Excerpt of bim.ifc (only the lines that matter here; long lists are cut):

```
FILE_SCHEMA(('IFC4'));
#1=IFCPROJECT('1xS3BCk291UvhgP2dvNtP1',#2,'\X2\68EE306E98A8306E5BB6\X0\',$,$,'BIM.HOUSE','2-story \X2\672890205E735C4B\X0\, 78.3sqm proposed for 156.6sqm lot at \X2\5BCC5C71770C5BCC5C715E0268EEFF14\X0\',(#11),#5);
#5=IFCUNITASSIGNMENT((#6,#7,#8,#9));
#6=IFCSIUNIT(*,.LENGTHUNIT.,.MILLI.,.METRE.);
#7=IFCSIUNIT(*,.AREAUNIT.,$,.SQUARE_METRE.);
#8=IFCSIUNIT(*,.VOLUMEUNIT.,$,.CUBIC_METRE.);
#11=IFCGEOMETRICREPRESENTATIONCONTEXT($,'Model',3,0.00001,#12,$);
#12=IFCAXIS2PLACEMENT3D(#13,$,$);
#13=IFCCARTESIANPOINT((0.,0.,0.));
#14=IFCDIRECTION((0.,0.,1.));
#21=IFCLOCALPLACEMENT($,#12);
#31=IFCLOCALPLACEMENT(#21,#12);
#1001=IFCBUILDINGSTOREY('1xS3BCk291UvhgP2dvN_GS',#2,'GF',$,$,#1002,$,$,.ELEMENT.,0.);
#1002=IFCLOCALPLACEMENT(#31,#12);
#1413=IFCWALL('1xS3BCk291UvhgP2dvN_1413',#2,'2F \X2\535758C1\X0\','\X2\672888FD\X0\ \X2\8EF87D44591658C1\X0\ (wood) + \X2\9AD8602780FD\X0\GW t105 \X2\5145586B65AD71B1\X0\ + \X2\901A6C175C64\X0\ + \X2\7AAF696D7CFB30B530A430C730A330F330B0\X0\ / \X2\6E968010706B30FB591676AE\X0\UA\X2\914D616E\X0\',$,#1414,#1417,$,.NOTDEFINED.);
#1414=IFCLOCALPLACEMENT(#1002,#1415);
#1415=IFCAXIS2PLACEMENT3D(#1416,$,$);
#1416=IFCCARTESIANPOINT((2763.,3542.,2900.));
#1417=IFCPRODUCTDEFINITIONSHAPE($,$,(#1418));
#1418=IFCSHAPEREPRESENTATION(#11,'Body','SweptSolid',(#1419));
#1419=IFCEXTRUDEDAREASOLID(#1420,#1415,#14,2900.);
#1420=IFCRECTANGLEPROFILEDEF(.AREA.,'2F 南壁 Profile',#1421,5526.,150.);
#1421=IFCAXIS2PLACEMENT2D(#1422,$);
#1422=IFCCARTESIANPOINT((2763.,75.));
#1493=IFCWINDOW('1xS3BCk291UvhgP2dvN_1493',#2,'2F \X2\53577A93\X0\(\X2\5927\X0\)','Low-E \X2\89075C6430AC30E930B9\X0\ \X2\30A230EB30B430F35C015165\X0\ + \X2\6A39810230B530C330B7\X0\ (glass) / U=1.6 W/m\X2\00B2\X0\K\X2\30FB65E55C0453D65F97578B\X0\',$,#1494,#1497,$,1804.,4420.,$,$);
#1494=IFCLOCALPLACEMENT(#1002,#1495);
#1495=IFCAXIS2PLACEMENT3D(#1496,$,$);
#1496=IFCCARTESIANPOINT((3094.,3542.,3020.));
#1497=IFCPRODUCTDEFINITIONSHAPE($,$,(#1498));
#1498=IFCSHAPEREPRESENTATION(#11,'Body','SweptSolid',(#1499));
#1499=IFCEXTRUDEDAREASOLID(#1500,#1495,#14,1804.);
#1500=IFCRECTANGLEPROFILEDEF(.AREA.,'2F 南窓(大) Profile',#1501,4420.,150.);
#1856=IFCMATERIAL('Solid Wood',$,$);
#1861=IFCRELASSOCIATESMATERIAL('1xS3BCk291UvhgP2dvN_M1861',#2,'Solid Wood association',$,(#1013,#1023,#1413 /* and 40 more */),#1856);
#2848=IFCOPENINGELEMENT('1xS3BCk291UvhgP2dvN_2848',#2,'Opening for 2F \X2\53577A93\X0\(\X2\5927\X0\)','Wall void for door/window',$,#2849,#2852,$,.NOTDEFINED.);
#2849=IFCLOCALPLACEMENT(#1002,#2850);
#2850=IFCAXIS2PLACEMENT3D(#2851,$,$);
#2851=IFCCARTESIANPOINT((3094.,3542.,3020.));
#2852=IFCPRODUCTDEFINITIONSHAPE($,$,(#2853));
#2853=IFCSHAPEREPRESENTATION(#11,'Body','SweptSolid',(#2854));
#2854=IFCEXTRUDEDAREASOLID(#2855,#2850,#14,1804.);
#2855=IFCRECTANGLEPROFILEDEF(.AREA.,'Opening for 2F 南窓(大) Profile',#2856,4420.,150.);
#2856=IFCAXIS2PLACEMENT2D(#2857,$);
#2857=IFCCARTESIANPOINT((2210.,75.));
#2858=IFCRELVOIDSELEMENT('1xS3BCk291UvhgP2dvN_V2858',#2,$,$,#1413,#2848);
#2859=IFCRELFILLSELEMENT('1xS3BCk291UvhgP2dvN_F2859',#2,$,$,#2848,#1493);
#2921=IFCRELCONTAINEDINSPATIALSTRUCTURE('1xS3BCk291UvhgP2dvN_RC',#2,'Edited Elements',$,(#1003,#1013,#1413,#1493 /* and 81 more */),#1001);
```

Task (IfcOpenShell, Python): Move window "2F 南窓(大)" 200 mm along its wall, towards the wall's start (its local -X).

```python
import ifcopenshell
import ifcopenshell.api.geometry
import ifcopenshell.util.placement

model = ifcopenshell.open("bim.ifc")

window = model.by_guid("1xS3BCk291UvhgP2dvN_1493")
opening = window.FillsVoids[0].RelatingOpeningElement
wall = opening.VoidsElements[0].RelatingBuildingElement

wall_matrix = ifcopenshell.util.placement.get_local_placement(wall.ObjectPlacement)
shift = wall_matrix[:3, 0] * -200.0
before = ifcopenshell.util.placement.get_local_placement(window.ObjectPlacement)[:3, 3].copy()

# The window is not placed relative to its opening, so move both.
for product in (opening, window):
    matrix = ifcopenshell.util.placement.get_local_placement(product.ObjectPlacement)
    matrix[:3, 3] += shift
    ifcopenshell.api.geometry.edit_object_placement(model, product=product, matrix=matrix, is_si=False)

after = ifcopenshell.util.placement.get_local_placement(window.ObjectPlacement)[:3, 3]
print("window moved by", (after - before).round(3) + 0.0)

model.write("bim_updated.ifc")
```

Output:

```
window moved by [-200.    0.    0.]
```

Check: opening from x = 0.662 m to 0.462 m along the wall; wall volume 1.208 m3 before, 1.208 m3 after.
